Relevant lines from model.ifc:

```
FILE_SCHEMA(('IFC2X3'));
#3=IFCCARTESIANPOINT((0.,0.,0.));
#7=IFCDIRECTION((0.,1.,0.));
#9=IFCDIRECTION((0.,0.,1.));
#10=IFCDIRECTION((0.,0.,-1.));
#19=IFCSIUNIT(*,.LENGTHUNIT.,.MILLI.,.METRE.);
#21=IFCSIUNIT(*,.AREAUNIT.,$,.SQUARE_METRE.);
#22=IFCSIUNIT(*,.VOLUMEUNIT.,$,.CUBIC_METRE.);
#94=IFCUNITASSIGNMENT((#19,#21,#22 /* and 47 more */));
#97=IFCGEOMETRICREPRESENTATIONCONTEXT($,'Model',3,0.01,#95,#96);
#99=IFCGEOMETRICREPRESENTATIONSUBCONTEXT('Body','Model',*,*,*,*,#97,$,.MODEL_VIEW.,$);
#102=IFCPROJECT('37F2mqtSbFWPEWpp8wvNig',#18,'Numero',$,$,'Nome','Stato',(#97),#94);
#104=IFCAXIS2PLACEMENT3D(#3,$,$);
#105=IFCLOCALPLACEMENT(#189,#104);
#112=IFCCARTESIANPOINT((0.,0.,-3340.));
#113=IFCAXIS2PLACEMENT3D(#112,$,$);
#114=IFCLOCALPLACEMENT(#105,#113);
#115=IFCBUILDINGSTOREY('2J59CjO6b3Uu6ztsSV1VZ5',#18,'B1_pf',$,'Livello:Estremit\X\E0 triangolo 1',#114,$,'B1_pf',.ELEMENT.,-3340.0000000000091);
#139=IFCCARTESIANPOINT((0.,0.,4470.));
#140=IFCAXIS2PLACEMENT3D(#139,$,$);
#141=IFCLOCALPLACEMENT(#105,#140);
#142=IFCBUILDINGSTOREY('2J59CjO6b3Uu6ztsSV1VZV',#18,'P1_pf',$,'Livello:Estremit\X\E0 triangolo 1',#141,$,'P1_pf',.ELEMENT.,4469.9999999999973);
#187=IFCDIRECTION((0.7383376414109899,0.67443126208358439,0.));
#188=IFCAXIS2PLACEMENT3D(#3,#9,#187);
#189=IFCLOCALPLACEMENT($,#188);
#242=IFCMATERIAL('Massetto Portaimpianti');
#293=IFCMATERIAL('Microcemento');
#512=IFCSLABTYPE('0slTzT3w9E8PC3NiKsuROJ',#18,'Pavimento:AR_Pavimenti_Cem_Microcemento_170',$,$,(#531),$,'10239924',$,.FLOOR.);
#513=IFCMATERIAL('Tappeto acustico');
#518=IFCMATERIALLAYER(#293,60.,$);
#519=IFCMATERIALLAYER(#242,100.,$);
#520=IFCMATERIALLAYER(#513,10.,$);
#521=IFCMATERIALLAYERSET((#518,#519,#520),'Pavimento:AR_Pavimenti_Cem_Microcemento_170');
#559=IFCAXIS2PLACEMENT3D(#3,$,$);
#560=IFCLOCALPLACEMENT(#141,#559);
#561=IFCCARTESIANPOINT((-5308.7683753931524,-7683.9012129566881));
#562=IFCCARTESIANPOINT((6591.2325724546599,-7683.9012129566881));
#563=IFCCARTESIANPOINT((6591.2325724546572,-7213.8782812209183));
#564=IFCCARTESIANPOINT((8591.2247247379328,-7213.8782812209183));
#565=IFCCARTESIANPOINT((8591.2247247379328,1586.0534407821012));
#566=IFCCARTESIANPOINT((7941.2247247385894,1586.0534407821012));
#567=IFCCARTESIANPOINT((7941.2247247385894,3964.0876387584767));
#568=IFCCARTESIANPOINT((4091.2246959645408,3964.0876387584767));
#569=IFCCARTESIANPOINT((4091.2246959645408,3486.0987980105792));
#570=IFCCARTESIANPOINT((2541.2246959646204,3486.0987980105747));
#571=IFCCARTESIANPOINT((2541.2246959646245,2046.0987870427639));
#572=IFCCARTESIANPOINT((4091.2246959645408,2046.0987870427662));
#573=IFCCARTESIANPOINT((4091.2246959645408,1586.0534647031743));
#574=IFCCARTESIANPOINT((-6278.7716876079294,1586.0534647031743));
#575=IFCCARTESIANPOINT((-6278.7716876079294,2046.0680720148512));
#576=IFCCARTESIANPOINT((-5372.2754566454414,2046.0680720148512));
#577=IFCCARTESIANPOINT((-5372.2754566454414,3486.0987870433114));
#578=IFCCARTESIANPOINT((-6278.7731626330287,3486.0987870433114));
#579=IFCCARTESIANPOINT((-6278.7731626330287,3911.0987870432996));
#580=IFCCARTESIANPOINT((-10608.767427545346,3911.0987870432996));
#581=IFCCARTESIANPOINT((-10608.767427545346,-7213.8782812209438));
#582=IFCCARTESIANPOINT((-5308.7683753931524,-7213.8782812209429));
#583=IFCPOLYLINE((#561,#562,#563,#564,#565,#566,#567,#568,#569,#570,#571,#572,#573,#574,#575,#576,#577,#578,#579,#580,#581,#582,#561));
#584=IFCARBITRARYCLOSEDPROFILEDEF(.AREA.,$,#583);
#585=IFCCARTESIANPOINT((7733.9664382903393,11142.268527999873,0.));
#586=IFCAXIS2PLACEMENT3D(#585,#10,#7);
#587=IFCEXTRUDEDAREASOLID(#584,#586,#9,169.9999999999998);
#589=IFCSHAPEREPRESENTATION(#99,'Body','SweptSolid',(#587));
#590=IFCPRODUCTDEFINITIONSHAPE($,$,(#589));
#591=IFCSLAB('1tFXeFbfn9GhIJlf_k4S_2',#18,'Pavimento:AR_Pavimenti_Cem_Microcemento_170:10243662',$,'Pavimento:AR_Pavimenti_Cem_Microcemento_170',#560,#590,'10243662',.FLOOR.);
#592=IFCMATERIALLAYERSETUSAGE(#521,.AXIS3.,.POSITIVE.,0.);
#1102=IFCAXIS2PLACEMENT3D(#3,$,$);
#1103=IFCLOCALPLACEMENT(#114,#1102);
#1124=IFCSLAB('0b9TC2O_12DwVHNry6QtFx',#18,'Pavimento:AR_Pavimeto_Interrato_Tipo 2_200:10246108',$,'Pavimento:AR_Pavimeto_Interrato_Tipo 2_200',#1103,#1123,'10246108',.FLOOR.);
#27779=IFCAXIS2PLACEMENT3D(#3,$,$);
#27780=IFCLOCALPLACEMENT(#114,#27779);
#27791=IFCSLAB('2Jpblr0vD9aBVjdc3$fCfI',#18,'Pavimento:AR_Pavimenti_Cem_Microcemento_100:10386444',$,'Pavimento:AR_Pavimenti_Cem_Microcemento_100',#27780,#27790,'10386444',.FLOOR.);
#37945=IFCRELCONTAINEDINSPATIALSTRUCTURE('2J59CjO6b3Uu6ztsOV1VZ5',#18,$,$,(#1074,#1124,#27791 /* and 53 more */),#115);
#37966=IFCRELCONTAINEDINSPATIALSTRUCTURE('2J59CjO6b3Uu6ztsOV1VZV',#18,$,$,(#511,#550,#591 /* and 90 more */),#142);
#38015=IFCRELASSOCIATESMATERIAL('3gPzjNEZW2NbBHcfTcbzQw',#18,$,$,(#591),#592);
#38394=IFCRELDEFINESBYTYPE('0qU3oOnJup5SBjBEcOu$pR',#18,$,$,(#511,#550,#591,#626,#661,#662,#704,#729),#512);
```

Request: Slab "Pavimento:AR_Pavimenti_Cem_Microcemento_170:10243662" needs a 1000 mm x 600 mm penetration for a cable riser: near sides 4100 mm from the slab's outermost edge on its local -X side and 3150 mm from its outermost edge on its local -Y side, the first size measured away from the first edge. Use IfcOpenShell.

```python
import numpy as np
import ifcopenshell
import ifcopenshell.api.feature
import ifcopenshell.api.geometry
import ifcopenshell.api.root
import ifcopenshell.geom
import ifcopenshell.util.placement
import ifcopenshell.util.representation
import ifcopenshell.util.shape
import ifcopenshell.util.unit

model = ifcopenshell.open("model.ifc")
unit_scale = ifcopenshell.util.unit.calculate_unit_scale(model)
settings = ifcopenshell.geom.settings()


def volume(element):
    """Net volume in cubic metres, openings subtracted."""
    shape = ifcopenshell.geom.create_shape(settings, element)
    return ifcopenshell.util.shape.get_volume(shape.geometry)


slab = model.by_guid("1tFXeFbfn9GhIJlf_k4S_2")
before = volume(slab)

# Extent in the slab's own axes, in metres. The edges named are its -X and -Y sides.
slab_shape = ifcopenshell.geom.create_shape(settings, slab)
vertices = ifcopenshell.util.shape.get_vertices(slab_shape.geometry)
x_min, y_min, bottom = vertices.min(axis=0)
top = vertices[:, 2].max()

opening = ifcopenshell.api.root.create_entity(model, ifc_class="IfcOpeningElement", name="Cable riser opening")
context = ifcopenshell.util.representation.get_context(model, "Model", "Body", "MODEL_VIEW")
width, depth = 1, 0.6
outline = [(0.0, 0.0), (width, 0.0), (width, depth), (0.0, depth), (0.0, 0.0)]
# Overshoot both faces by 50 mm so the cut is clean.
shape = ifcopenshell.api.geometry.add_slab_representation(
    model, context=context, depth=top - bottom + 0.1, polyline=outline
)
ifcopenshell.api.geometry.assign_representation(model, product=opening, representation=shape)

matrix = ifcopenshell.util.placement.get_local_placement(slab.ObjectPlacement)
matrix[:, 3] = matrix @ np.append(np.array([x_min + 4.1, y_min + 3.15, bottom - 0.05]) / unit_scale, 1.0)
ifcopenshell.api.geometry.edit_object_placement(model, product=opening, matrix=matrix, is_si=False)
ifcopenshell.api.feature.add_feature(model, feature=opening, element=slab)

after = volume(slab)

print(f"slab volume {before:.3f} -> {after:.3f} m3")

model.write("model_rev.ifc")
```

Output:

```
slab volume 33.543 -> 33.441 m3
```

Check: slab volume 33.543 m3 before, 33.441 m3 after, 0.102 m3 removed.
